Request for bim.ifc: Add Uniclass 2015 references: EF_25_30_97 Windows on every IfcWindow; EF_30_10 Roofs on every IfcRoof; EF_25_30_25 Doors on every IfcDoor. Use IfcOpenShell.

First a look at what the model holds.

```python
import ifcopenshell

model = ifcopenshell.open("bim.ifc")
print(model.schema)
print("classifications:", [c.Name for c in model.by_type("IfcClassification")])
for ifc_class in ("IfcDoor", "IfcRoof", "IfcStair", "IfcWall", "IfcWindow"):
    print(ifc_class, len(model.by_type(ifc_class)))
```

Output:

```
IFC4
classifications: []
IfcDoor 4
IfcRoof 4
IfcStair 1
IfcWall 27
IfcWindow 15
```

```python
import ifcopenshell
import ifcopenshell.api.classification

model = ifcopenshell.open("bim.ifc")

system = ifcopenshell.api.classification.add_classification(model, classification="Uniclass 2015")

codes = {
    "IfcWindow": ("EF_25_30_97", "Windows"),
    "IfcRoof": ("EF_30_10", "Roofs"),
    "IfcDoor": ("EF_25_30_25", "Doors"),
}
for ifc_class, (code, name) in codes.items():
    products = model.by_type(ifc_class)
    ifcopenshell.api.classification.add_reference(
        model, products=products, classification=system, identification=code, name=name
    )
    print(code, len(products))

model.write("bim_rev.ifc")
```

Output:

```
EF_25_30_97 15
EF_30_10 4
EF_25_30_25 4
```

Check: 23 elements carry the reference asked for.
